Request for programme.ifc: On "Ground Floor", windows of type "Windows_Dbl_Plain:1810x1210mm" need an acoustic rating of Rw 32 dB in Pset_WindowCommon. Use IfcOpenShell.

First a look at what the model holds.

```python
import ifcopenshell
import ifcopenshell.util.element

model = ifcopenshell.open("programme.ifc")
print(model.schema)
storey = next(s for s in model.by_type("IfcBuildingStorey") if s.Name == "Ground Floor")
windows = [e for e in ifcopenshell.util.element.get_decomposition(storey) if e.is_a("IfcWindow")]
seen = {}
for e in windows:
    element_type = ifcopenshell.util.element.get_type(e)
    key = (element_type.Name if element_type != e and element_type else None, ifcopenshell.util.element.get_pset(e, "Pset_WindowCommon", "AcousticRating"))
    seen[key] = seen.get(key, 0) + 1
for (name, value), count in sorted(seen.items(), key=str):
    print(count, "x", name, "|", value)
```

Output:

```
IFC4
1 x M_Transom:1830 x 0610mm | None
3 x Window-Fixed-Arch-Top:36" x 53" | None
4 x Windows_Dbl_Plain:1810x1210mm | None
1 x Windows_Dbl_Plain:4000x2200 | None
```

```python
import ifcopenshell
import ifcopenshell.api.pset
import ifcopenshell.util.element

model = ifcopenshell.open("programme.ifc")

storey = next(s for s in model.by_type("IfcBuildingStorey") if s.Name == "Ground Floor")
windows = [e for e in ifcopenshell.util.element.get_decomposition(storey) if e.is_a("IfcWindow")]

count = 0
for e in windows:
    element_type = ifcopenshell.util.element.get_type(e)
    if element_type in (None, e) or element_type.Name != "Windows_Dbl_Plain:1810x1210mm":
        continue
    # add_pset returns the element's existing set when there is one.
    pset = ifcopenshell.api.pset.add_pset(model, product=e, name="Pset_WindowCommon")
    ifcopenshell.api.pset.edit_pset(model, pset=pset, properties={"AcousticRating": "Rw 32 dB"})
    count += 1

print(count, "windows updated")

model.write("programme_rev.ifc")
```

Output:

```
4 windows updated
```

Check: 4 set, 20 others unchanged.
